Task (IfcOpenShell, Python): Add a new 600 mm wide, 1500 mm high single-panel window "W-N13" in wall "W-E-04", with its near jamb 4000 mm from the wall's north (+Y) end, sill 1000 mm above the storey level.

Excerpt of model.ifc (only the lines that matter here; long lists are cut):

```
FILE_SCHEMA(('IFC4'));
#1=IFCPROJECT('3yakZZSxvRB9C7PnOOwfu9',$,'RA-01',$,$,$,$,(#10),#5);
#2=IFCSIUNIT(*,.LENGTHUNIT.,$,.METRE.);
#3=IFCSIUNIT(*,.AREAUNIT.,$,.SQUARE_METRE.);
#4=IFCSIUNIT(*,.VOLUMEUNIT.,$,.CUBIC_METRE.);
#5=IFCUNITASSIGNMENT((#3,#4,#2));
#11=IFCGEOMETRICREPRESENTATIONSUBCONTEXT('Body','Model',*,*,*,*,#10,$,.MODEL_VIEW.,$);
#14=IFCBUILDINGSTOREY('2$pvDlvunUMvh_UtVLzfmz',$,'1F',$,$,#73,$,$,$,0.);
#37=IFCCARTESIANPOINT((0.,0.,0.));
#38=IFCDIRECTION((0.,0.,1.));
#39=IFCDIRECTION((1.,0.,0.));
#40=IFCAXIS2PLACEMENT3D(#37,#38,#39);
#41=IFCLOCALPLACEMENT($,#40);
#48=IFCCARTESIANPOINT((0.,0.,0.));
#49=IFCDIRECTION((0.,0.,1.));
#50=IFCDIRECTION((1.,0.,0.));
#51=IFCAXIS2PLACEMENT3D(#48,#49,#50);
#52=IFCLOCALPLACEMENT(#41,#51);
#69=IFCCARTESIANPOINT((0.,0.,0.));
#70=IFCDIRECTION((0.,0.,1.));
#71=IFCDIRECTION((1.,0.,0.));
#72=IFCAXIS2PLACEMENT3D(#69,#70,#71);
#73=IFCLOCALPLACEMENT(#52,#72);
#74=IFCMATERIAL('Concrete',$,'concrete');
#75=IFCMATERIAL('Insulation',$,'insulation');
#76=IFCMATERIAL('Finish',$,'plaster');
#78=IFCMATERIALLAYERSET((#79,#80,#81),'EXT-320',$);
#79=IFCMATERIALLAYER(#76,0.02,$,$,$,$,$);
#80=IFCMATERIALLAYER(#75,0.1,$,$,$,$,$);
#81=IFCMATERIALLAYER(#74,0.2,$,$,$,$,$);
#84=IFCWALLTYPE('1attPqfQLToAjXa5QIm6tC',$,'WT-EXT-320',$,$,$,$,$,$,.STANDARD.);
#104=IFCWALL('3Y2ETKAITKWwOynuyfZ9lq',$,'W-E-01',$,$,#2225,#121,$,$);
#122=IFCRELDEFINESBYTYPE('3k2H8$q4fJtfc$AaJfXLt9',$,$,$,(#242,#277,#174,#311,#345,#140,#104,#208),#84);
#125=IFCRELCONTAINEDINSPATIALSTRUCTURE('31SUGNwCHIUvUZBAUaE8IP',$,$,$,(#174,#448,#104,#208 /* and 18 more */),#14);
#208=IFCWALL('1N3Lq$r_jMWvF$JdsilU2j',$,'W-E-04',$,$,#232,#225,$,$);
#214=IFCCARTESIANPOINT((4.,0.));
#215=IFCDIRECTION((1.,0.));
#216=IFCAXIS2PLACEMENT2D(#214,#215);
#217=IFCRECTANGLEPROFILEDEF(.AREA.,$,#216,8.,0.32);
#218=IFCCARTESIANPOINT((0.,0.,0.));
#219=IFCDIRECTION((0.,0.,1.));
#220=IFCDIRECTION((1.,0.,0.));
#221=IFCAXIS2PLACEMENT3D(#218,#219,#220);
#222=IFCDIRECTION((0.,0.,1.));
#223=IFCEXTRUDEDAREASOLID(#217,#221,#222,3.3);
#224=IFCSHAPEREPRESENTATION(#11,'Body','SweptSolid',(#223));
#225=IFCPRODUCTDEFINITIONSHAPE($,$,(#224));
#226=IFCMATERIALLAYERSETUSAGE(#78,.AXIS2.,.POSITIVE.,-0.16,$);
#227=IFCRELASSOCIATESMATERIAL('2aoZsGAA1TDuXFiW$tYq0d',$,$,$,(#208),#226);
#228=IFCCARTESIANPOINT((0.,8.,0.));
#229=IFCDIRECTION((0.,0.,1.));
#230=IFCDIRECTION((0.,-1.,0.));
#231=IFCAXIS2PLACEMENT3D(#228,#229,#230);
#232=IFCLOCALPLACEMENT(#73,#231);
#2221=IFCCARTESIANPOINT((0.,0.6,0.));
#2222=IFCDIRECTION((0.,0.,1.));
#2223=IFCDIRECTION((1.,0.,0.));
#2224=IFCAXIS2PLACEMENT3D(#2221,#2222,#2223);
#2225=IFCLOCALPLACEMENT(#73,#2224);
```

```python
import numpy as np
import ifcopenshell
import ifcopenshell.api.feature
import ifcopenshell.api.geometry
import ifcopenshell.api.root
import ifcopenshell.api.spatial
import ifcopenshell.geom
import ifcopenshell.util.element
import ifcopenshell.util.placement
import ifcopenshell.util.representation
import ifcopenshell.util.shape
import ifcopenshell.util.unit

model = ifcopenshell.open("model.ifc")
unit_scale = ifcopenshell.util.unit.calculate_unit_scale(model)
settings = ifcopenshell.geom.settings()


def volume(element):
    """Net volume in cubic metres, openings subtracted."""
    shape = ifcopenshell.geom.create_shape(settings, element)
    return ifcopenshell.util.shape.get_volume(shape.geometry)


wall = model.by_guid("1N3Lq$r_jMWvF$JdsilU2j")
storey = ifcopenshell.util.element.get_container(wall, ifc_class="IfcBuildingStorey")
context = ifcopenshell.util.representation.get_context(model, "Model", "Body", "MODEL_VIEW")
before = volume(wall)

width, height, from_end, sill = 0.6, 1.5, 4, 1  # metres

# The wall runs along its own X axis, and the end named is its -X end.
wall_shape = ifcopenshell.geom.create_shape(settings, wall)
x, y, z = ifcopenshell.util.shape.get_vertices(wall_shape.geometry).T
start = x.min() + from_end
face, thickness = float(y.min()), float(y.max() - y.min())
wall_matrix = ifcopenshell.util.placement.get_local_placement(wall.ObjectPlacement)
level = ifcopenshell.util.placement.get_local_placement(storey.ObjectPlacement)[2, 3]


def in_wall(x, y):
    """Placement at x, y metres in the wall's axes, at sill height."""
    matrix = wall_matrix.copy()
    matrix[:, 3] = wall_matrix @ np.array([x / unit_scale, y / unit_scale, 0.0, 1.0])
    matrix[2, 3] = level + sill / unit_scale
    return matrix


# Opening: a box that overshoots both wall faces by 50 mm.
opening = ifcopenshell.api.root.create_entity(model, ifc_class="IfcOpeningElement", predefined_type="OPENING")
box = ifcopenshell.api.geometry.add_wall_representation(
    model, context=context, length=width, height=height, thickness=thickness + 0.1
)
ifcopenshell.api.geometry.assign_representation(model, product=opening, representation=box)
ifcopenshell.api.geometry.edit_object_placement(model, product=opening, matrix=in_wall(start, face - 0.05), is_si=False)
ifcopenshell.api.feature.add_feature(model, feature=opening, element=wall)

window = ifcopenshell.api.root.create_entity(model, ifc_class="IfcWindow", name="W-N13", predefined_type="WINDOW")
window.OverallWidth, window.OverallHeight = width / unit_scale, height / unit_scale
window.PartitioningType = "SINGLE_PANEL"
body = ifcopenshell.api.geometry.add_window_representation(
    model,
    context=context,
    overall_width=window.OverallWidth,
    overall_height=window.OverallHeight,
    partition_type="SINGLE_PANEL",
)
ifcopenshell.api.geometry.assign_representation(model, product=window, representation=body)
ifcopenshell.api.spatial.assign_container(model, products=[window], relating_structure=storey)
ifcopenshell.api.feature.add_filling(model, opening=opening, element=window)

# Centre the window in the wall's thickness.
ifcopenshell.api.geometry.edit_object_placement(model, product=window, matrix=in_wall(start, face), is_si=False)
window_shape = ifcopenshell.geom.create_shape(settings, window)
depth = ifcopenshell.util.shape.get_vertices(window_shape.geometry)[:, 1]
offset = face + thickness / 2 - (depth.min() + depth.max()) / 2
ifcopenshell.api.geometry.edit_object_placement(model, product=window, matrix=in_wall(start, offset), is_si=False)

after = volume(wall)

print(f"wall volume {before:.3f} -> {after:.3f} m3")

model.write("model-out.ifc")
```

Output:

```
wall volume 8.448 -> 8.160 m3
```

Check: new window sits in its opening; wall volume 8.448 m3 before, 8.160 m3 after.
